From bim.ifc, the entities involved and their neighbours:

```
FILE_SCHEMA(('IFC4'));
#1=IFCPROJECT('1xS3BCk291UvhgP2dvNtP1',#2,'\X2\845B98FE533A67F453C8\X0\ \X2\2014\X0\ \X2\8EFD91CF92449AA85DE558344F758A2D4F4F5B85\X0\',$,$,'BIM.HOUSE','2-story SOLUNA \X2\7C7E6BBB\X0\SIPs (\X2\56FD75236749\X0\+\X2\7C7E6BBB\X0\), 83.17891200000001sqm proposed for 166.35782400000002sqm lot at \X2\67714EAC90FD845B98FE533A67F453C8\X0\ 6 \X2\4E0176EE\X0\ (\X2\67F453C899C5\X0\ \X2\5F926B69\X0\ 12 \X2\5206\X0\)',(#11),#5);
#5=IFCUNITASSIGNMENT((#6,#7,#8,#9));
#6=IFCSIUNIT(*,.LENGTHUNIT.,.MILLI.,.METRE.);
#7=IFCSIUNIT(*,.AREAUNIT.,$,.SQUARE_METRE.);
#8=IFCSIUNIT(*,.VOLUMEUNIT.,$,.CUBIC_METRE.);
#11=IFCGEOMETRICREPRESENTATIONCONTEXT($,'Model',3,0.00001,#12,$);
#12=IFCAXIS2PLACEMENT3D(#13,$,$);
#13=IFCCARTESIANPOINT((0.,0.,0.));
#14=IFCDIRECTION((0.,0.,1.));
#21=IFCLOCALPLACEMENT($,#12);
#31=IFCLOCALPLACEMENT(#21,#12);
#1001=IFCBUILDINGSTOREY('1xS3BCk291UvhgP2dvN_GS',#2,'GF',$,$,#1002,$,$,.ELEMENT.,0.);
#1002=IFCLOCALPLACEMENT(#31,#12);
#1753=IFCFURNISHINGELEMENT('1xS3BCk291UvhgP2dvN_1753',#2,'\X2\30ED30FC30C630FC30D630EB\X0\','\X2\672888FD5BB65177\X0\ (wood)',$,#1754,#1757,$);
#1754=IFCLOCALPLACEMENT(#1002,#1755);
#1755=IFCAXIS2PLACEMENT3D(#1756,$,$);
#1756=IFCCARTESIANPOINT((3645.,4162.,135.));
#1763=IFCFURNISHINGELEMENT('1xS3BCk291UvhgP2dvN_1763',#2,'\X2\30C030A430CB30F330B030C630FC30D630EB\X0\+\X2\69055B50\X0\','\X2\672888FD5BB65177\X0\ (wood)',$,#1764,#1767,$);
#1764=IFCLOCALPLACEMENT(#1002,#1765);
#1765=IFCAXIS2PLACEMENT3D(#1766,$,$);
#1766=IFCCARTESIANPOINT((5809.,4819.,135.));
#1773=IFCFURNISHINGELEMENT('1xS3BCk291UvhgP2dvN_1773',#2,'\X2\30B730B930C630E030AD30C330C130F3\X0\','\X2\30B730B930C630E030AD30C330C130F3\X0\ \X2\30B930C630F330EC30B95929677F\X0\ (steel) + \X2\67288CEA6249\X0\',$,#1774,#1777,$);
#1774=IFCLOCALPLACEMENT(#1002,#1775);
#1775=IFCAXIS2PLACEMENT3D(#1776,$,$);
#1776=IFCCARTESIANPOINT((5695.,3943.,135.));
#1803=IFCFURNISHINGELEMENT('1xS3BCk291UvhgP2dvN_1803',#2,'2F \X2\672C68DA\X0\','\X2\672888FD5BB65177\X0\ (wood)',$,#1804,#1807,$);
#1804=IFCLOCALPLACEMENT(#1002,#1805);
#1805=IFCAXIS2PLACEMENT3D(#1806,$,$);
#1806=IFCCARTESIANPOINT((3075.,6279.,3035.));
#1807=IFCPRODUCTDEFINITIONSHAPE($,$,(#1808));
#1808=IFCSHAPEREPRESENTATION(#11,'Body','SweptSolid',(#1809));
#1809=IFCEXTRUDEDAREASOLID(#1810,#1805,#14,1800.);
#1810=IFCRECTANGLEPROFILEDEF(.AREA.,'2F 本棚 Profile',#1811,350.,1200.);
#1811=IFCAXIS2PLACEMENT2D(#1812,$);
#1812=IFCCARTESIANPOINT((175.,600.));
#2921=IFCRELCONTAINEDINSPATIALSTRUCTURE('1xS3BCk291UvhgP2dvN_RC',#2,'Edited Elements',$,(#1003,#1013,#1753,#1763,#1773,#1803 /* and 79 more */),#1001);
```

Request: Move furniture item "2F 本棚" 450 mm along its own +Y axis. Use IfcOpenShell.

```python
import ifcopenshell
import ifcopenshell.api.geometry
import ifcopenshell.util.placement
import ifcopenshell.util.unit

model = ifcopenshell.open("bim.ifc")
unit_scale = ifcopenshell.util.unit.calculate_unit_scale(model)

item = model.by_guid("1xS3BCk291UvhgP2dvN_1803")
matrix = ifcopenshell.util.placement.get_local_placement(item.ObjectPlacement)
matrix[:3, 3] += matrix[:3, 1] * 0.45 / unit_scale
ifcopenshell.api.geometry.edit_object_placement(model, product=item, matrix=matrix, is_si=False)

print(ifcopenshell.util.placement.get_local_placement(item.ObjectPlacement).round(3) + 0.0)

model.write("bim_edited.ifc")
```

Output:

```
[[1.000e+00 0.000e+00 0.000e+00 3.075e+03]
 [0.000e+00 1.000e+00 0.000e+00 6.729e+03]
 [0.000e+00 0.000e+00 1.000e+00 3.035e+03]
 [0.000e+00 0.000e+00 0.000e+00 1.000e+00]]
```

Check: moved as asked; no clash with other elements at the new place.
